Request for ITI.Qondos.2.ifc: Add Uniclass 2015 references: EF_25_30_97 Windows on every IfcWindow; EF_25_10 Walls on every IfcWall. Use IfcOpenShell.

First a look at what the model holds.

```python
import ifcopenshell

model = ifcopenshell.open("ITI.Qondos.2.ifc")
print(model.schema)
print("classifications:", [c.Name for c in model.by_type("IfcClassification")])
for ifc_class in ("IfcDoor", "IfcRoof", "IfcStair", "IfcWall", "IfcWindow"):
    print(ifc_class, len(model.by_type(ifc_class)))
```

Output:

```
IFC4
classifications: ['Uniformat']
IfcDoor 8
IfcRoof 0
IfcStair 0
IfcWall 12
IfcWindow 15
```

```python
import ifcopenshell
import ifcopenshell.api.classification

model = ifcopenshell.open("ITI.Qondos.2.ifc")

system = ifcopenshell.api.classification.add_classification(model, classification="Uniclass 2015")

codes = {
    "IfcWindow": ("EF_25_30_97", "Windows"),
    "IfcWall": ("EF_25_10", "Walls"),
}
for ifc_class, (code, name) in codes.items():
    products = model.by_type(ifc_class)
    ifcopenshell.api.classification.add_reference(
        model, products=products, classification=system, identification=code, name=name
    )
    print(code, len(products))

model.write("ITI.Qondos.2_v2.ifc")
```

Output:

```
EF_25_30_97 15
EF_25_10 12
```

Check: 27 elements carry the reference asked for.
